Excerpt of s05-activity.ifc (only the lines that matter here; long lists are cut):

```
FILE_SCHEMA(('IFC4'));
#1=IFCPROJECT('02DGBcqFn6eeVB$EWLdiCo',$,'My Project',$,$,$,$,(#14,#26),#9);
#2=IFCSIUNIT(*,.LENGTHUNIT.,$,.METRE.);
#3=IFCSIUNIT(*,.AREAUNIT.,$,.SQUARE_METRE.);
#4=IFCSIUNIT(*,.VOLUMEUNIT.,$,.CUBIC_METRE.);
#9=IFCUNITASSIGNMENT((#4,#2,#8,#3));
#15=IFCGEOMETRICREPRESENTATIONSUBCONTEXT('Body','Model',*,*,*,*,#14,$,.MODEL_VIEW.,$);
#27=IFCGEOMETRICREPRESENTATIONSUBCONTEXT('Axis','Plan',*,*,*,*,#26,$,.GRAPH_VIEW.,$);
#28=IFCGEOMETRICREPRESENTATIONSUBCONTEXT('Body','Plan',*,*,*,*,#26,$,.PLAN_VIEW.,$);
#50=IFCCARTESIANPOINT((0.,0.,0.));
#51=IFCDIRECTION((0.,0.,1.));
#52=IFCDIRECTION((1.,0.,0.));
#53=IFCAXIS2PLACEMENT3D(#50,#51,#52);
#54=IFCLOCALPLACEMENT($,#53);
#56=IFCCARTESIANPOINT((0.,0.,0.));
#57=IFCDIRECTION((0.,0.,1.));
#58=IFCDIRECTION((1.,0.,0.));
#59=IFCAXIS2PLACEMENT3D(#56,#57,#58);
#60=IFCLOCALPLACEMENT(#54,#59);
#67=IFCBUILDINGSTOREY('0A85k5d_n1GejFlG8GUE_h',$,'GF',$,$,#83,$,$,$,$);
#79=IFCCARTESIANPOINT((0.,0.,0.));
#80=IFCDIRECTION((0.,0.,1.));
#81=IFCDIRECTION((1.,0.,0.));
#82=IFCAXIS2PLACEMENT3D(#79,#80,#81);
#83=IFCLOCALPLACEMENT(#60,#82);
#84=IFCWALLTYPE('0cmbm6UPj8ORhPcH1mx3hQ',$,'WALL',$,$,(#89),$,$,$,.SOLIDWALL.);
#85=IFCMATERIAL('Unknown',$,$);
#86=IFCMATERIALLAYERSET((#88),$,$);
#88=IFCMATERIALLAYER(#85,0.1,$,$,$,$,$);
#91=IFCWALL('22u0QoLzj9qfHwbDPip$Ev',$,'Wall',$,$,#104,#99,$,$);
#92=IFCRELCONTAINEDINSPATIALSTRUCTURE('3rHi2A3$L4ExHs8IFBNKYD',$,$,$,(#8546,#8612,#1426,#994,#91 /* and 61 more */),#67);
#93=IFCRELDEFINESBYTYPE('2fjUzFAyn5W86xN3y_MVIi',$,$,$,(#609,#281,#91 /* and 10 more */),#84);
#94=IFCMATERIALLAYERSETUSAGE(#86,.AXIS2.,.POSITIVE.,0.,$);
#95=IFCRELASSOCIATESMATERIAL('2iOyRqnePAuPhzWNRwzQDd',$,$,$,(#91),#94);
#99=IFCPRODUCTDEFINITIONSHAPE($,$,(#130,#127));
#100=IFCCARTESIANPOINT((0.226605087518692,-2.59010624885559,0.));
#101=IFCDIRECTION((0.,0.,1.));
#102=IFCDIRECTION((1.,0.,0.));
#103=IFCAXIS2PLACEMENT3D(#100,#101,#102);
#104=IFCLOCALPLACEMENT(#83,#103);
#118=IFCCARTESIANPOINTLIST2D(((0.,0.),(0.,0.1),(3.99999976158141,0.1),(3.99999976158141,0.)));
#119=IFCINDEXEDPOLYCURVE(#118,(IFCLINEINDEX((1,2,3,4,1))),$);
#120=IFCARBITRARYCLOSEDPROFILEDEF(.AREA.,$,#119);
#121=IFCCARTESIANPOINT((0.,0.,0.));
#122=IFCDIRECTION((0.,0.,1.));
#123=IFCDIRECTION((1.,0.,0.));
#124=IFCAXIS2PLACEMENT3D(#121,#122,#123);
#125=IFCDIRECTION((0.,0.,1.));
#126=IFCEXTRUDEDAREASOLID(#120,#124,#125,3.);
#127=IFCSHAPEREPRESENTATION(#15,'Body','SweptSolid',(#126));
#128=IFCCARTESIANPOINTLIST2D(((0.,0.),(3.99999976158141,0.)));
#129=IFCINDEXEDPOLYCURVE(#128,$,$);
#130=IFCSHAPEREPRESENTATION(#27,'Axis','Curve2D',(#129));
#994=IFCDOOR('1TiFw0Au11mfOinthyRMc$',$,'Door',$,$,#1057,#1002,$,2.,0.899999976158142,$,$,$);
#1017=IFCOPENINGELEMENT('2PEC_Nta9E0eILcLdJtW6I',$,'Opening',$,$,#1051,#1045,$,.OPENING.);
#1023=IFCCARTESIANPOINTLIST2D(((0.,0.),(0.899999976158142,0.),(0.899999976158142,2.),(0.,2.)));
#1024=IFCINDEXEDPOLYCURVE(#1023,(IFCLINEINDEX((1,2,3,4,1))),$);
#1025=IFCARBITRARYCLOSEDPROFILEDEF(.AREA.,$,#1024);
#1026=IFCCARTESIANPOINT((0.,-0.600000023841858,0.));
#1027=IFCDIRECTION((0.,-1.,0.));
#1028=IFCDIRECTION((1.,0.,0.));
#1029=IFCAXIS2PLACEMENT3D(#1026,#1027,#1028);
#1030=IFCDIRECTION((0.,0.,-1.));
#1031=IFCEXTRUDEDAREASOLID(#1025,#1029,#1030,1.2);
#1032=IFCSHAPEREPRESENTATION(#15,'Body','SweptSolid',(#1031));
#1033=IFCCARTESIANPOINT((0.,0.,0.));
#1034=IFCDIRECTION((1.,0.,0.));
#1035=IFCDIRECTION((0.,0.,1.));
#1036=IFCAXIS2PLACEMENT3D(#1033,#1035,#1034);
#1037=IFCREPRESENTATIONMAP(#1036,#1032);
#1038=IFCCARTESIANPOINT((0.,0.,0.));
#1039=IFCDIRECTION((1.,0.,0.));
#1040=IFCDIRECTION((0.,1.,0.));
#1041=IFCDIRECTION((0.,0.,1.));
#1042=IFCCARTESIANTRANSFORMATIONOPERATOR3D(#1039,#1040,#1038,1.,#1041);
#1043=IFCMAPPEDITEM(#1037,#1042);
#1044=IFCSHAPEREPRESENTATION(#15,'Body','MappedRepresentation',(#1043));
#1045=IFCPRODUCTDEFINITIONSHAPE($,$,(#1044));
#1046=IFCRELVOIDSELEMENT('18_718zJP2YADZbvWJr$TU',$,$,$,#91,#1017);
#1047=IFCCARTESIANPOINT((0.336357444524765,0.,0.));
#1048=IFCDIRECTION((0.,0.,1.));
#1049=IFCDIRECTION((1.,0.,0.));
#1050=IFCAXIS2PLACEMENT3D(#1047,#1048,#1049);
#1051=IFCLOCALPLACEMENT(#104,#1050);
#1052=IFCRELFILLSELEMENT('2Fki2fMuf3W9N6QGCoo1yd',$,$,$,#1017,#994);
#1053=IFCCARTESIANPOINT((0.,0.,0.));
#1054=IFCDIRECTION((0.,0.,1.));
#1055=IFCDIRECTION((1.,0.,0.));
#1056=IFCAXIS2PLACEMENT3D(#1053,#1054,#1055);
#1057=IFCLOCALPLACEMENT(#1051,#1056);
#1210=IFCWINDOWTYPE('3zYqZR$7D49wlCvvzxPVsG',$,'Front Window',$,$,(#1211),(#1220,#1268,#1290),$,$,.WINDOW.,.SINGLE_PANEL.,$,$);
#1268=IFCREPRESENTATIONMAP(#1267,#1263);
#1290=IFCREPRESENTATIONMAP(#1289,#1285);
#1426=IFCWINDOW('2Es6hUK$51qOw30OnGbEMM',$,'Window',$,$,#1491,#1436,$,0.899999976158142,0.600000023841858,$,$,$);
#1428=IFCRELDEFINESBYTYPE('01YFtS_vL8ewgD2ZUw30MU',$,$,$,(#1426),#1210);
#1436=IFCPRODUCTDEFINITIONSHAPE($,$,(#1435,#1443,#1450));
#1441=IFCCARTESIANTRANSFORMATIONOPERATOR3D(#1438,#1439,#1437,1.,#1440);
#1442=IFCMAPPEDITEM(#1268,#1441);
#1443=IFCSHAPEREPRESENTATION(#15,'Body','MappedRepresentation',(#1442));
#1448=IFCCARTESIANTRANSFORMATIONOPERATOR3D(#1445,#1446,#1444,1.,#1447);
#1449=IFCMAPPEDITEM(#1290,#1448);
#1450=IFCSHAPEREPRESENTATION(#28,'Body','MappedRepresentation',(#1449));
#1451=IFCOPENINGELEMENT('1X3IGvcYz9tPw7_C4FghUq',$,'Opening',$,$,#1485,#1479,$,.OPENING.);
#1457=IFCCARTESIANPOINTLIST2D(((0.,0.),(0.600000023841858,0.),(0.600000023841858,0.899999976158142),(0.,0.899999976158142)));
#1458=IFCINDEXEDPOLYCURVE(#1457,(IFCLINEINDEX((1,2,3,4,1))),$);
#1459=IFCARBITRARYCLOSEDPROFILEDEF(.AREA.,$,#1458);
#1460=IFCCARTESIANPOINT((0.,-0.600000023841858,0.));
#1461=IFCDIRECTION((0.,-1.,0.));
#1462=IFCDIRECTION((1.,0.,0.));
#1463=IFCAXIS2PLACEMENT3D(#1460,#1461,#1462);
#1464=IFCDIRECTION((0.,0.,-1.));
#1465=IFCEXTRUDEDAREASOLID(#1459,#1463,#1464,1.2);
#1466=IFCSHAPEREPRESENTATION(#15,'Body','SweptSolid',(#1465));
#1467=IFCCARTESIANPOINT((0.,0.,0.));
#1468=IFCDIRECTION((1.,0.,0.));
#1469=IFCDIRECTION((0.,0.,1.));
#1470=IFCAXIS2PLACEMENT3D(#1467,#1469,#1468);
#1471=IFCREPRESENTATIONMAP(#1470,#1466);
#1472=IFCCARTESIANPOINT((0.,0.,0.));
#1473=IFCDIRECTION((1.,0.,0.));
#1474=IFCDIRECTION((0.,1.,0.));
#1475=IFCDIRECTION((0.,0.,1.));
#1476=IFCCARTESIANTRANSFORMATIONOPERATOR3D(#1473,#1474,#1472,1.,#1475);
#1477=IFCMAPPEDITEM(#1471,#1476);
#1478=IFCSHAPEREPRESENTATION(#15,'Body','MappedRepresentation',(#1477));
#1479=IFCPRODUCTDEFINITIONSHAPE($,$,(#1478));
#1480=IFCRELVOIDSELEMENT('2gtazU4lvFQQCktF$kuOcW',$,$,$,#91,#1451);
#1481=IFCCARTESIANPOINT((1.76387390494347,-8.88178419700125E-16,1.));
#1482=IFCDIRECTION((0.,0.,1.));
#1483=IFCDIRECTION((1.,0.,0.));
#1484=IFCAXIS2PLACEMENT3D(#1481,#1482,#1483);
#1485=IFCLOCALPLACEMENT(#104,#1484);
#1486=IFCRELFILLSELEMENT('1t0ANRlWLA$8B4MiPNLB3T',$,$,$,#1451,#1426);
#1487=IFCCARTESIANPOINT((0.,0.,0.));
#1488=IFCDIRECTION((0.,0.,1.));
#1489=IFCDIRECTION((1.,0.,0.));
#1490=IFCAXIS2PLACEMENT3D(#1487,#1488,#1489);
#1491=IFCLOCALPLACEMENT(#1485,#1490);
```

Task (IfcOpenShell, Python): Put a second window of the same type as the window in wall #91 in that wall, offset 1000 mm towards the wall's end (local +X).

```python
import ifcopenshell
import ifcopenshell.api.feature
import ifcopenshell.api.geometry
import ifcopenshell.api.root
import ifcopenshell.geom
import ifcopenshell.util.element
import ifcopenshell.util.placement
import ifcopenshell.util.shape

model = ifcopenshell.open("s05-activity.ifc")
settings = ifcopenshell.geom.settings()


def volume(element):
    """Net volume in cubic metres, openings subtracted."""
    shape = ifcopenshell.geom.create_shape(settings, element)
    return ifcopenshell.util.shape.get_volume(shape.geometry)


window = model.by_guid("2Es6hUK$51qOw30OnGbEMM")
opening = window.FillsVoids[0].RelatingOpeningElement
wall = opening.VoidsElements[0].RelatingBuildingElement
before = volume(wall)
shift = ifcopenshell.util.placement.get_local_placement(wall.ObjectPlacement)[:3, 0] * 1.0

# copy_class copies the void relationship, type, container and properties, but no geometry.
new_opening = ifcopenshell.api.root.copy_class(model, product=opening)
new_opening.Representation = ifcopenshell.util.element.copy_deep(
    model, opening.Representation, exclude=["IfcGeometricRepresentationContext", "IfcRepresentationMap"]
)
new_window = ifcopenshell.api.root.copy_class(model, product=window)
new_window.Representation = ifcopenshell.util.element.copy_deep(
    model, window.Representation, exclude=["IfcGeometricRepresentationContext", "IfcRepresentationMap"]
)
ifcopenshell.api.feature.add_filling(model, opening=new_opening, element=new_window)

for old, new in ((opening, new_opening), (window, new_window)):
    matrix = ifcopenshell.util.placement.get_local_placement(old.ObjectPlacement)
    matrix[:3, 3] += shift
    ifcopenshell.api.geometry.edit_object_placement(model, product=new, matrix=matrix, is_si=False)

after = volume(wall)

print(f"wall volume {before:.3f} -> {after:.3f} m3")

model.write("s05-activity_rev.ifc")
```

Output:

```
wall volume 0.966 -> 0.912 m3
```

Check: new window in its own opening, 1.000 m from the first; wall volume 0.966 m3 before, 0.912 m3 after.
